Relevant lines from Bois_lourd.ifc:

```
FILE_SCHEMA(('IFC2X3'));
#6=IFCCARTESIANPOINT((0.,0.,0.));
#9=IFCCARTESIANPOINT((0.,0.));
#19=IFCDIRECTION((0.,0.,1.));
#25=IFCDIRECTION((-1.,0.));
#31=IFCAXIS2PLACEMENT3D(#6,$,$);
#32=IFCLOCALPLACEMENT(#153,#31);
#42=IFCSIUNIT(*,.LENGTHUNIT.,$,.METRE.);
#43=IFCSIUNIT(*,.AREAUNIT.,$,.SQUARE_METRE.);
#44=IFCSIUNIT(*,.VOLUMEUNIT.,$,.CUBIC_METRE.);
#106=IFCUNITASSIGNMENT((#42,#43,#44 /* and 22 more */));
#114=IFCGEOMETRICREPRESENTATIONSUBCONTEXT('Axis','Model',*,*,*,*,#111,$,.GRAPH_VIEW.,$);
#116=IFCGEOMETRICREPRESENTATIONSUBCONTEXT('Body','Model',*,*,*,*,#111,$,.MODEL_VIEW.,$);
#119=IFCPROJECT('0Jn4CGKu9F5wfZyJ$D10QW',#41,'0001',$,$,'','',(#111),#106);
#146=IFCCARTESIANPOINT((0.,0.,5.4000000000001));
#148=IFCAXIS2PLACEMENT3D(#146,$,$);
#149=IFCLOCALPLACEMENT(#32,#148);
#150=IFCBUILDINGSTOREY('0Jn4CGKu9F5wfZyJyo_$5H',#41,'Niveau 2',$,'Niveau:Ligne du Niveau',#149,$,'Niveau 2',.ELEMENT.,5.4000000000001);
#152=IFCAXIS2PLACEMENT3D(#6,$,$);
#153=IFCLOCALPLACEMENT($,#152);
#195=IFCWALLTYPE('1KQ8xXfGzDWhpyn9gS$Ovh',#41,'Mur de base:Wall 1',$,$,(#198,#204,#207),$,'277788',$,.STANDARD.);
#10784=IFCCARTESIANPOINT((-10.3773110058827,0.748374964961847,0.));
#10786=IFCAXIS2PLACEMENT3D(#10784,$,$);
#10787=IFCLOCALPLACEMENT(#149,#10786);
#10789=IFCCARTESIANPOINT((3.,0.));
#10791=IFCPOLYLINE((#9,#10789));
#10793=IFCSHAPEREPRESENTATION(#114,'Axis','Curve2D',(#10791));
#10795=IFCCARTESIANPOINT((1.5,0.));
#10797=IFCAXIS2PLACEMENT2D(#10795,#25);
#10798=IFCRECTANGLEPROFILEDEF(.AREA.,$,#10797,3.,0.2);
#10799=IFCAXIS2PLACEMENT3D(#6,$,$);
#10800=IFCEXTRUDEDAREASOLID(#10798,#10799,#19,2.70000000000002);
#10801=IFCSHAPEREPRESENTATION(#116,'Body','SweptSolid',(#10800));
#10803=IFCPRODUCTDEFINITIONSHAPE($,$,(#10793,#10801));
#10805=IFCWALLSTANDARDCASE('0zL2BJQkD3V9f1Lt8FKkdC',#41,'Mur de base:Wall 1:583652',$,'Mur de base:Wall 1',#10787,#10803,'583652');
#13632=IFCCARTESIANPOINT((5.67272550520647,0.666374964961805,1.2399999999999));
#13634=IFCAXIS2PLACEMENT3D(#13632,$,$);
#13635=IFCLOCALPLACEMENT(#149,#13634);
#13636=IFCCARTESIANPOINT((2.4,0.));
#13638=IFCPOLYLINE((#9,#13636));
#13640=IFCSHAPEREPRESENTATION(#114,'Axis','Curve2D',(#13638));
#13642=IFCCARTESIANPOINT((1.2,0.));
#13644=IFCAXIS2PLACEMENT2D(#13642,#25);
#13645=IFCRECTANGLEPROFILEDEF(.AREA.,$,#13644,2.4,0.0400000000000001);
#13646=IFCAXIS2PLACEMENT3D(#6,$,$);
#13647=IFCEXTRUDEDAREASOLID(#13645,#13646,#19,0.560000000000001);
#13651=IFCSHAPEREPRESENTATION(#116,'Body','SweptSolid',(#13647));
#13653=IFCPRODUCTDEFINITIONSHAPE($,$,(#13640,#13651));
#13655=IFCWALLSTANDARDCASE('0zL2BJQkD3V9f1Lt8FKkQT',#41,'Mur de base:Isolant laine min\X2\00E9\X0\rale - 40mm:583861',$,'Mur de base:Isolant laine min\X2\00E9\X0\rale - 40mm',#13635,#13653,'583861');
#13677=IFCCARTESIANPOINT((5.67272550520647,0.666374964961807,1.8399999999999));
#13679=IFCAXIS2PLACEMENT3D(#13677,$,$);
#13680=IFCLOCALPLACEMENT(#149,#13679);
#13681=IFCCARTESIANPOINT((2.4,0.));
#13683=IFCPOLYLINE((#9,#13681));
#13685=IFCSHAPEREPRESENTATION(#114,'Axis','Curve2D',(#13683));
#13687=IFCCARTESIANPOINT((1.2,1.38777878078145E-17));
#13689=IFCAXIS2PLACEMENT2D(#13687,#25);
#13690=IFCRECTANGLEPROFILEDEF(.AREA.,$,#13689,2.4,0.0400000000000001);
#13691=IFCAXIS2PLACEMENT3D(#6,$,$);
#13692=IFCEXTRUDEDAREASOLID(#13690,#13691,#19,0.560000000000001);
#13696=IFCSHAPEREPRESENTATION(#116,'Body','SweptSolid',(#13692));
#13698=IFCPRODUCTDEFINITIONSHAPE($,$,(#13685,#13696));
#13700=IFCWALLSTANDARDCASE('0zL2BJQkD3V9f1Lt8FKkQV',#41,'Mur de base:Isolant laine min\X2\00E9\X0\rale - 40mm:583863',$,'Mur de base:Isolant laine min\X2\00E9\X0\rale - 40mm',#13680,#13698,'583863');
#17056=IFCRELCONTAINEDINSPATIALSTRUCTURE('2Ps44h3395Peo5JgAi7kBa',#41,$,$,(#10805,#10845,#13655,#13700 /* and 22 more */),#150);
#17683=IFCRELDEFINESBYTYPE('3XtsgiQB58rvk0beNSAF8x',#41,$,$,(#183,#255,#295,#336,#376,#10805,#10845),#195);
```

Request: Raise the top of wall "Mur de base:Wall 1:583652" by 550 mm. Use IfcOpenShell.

```python
import ifcopenshell
import ifcopenshell.geom
import ifcopenshell.util.representation
import ifcopenshell.util.shape
import ifcopenshell.util.unit

model = ifcopenshell.open("Bois_lourd.ifc")
unit_scale = ifcopenshell.util.unit.calculate_unit_scale(model)
settings = ifcopenshell.geom.settings()


def volume(element):
    """Net volume in cubic metres, openings subtracted."""
    shape = ifcopenshell.geom.create_shape(settings, element)
    return ifcopenshell.util.shape.get_volume(shape.geometry)


wall = model.by_guid("0zL2BJQkD3V9f1Lt8FKkdC")
before = volume(wall)

body = ifcopenshell.util.representation.get_representation(wall, "Model", "Body")
solid = body.Items[0]
old_height = solid.Depth
solid.Depth += 0.55 / unit_scale
after = volume(wall)

print(f"height {old_height:g} -> {solid.Depth:g}, volume {before:.3f} -> {after:.3f} m3")

model.write("Bois_lourd-out.ifc")
```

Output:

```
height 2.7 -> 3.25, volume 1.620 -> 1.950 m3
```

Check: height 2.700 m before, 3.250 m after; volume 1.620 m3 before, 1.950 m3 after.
